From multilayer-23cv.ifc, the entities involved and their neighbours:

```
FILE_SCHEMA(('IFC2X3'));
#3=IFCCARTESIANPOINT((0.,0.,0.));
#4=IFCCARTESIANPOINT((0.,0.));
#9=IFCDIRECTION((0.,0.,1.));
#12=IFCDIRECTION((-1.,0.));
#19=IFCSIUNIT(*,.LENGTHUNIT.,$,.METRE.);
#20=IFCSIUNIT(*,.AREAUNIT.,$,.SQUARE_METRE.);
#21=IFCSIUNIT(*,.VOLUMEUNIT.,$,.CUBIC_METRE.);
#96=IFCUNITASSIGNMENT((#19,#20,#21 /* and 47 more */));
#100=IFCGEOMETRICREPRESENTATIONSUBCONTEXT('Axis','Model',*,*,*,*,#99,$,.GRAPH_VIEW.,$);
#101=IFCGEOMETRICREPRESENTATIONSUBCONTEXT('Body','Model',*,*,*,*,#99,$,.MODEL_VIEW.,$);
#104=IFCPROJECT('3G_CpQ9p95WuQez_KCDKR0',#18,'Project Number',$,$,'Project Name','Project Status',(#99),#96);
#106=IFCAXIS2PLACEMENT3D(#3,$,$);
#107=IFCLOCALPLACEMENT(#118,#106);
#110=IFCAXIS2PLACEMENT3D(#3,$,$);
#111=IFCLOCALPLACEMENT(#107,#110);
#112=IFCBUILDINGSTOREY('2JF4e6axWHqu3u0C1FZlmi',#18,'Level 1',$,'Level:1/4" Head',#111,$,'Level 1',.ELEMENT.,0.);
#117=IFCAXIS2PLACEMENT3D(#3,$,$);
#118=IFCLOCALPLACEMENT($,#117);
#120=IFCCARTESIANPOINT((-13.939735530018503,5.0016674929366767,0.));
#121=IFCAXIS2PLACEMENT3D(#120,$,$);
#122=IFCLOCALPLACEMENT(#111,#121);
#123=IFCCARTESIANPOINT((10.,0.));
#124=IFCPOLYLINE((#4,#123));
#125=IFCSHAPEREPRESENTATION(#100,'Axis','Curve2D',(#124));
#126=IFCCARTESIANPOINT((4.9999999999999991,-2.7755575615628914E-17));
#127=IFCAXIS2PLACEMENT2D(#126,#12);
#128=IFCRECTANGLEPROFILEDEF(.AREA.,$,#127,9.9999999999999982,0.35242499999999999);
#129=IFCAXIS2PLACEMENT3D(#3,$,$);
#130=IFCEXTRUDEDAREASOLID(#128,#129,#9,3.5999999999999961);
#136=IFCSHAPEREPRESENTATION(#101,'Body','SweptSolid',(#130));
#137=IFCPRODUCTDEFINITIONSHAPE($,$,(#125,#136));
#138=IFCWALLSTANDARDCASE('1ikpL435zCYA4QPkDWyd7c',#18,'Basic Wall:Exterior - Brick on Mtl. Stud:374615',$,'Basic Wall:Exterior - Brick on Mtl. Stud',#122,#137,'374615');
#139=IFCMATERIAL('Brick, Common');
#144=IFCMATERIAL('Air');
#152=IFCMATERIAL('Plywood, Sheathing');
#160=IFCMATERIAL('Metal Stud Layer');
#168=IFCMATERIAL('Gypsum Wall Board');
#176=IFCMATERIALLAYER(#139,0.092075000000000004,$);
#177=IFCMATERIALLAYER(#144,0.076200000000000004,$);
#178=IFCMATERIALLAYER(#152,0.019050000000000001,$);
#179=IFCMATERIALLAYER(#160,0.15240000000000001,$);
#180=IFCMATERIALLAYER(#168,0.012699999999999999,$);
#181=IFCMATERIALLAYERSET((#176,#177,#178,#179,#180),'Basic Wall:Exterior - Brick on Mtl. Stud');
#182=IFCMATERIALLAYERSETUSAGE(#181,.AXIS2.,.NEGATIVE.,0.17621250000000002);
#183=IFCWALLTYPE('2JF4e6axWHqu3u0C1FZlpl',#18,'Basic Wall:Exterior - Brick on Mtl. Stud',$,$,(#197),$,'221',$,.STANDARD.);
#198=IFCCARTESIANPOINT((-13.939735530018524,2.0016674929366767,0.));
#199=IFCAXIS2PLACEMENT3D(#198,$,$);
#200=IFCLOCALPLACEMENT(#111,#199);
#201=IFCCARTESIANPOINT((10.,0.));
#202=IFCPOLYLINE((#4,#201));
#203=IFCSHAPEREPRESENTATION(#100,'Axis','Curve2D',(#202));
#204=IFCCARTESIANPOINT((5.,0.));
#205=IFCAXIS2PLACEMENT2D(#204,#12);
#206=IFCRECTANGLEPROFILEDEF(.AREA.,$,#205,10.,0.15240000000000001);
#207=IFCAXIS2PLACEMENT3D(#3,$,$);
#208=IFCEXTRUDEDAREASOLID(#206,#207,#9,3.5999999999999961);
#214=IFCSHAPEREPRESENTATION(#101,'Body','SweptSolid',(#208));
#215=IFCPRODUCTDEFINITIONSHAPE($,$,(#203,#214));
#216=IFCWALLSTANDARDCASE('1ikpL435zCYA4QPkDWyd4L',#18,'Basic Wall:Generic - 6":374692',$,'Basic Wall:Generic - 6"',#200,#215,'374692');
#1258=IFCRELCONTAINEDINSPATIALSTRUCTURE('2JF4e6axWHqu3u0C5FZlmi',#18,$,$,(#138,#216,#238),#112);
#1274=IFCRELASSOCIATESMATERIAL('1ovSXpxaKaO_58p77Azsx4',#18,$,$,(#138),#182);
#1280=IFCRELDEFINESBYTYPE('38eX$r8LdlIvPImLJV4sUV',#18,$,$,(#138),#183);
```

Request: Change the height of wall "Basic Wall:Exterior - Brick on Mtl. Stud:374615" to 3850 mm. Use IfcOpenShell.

```python
import ifcopenshell
import ifcopenshell.geom
import ifcopenshell.util.representation
import ifcopenshell.util.shape
import ifcopenshell.util.unit

model = ifcopenshell.open("multilayer-23cv.ifc")
unit_scale = ifcopenshell.util.unit.calculate_unit_scale(model)
settings = ifcopenshell.geom.settings()


def volume(element):
    """Net volume in cubic metres, openings subtracted."""
    shape = ifcopenshell.geom.create_shape(settings, element)
    return ifcopenshell.util.shape.get_volume(shape.geometry)


wall = model.by_guid("1ikpL435zCYA4QPkDWyd7c")
before = volume(wall)

body = ifcopenshell.util.representation.get_representation(wall, "Model", "Body")
solid = body.Items[0]
old_height = solid.Depth
solid.Depth = 3.85 / unit_scale
after = volume(wall)

print(f"height {old_height:g} -> {solid.Depth:g}, volume {before:.3f} -> {after:.3f} m3")

model.write("multilayer-23cv_rev.ifc")
```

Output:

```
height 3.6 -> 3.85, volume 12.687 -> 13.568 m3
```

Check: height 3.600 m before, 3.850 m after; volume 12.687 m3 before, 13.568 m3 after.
